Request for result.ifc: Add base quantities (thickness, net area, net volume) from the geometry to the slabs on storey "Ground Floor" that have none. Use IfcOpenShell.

First a look at what the model holds.

```python
import ifcopenshell
import ifcopenshell.util.element
import ifcopenshell.util.unit

model = ifcopenshell.open("result.ifc")
print(model.schema)
for unit_type in ("LENGTHUNIT", "AREAUNIT", "VOLUMEUNIT"):
    print(unit_type, ifcopenshell.util.unit.calculate_unit_scale(model, unit_type))
storey = next(s for s in model.by_type("IfcBuildingStorey") if s.Name == "Ground Floor")
slabs = [e for e in ifcopenshell.util.element.get_decomposition(storey) if e.is_a("IfcSlab")]
for e in sorted(slabs, key=lambda e: e.id()):
    print(e.id(), e.is_a(), e.Name, list(ifcopenshell.util.element.get_psets(e, qtos_only=True)), sep=" | ")
```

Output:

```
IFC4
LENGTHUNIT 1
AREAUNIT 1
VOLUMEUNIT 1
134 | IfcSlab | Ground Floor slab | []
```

```python
import ifcopenshell
import ifcopenshell.api.pset
import ifcopenshell.geom
import ifcopenshell.util.element
import ifcopenshell.util.shape
import ifcopenshell.util.unit

model = ifcopenshell.open("result.ifc")
unit_scale = ifcopenshell.util.unit.calculate_unit_scale(model)
area_scale = ifcopenshell.util.unit.calculate_unit_scale(model, "AREAUNIT")
volume_scale = ifcopenshell.util.unit.calculate_unit_scale(model, "VOLUMEUNIT")
settings = ifcopenshell.geom.settings()

storey = next(s for s in model.by_type("IfcBuildingStorey") if s.Name == "Ground Floor")
slabs = [e for e in ifcopenshell.util.element.get_decomposition(storey) if e.is_a("IfcSlab")]

for e in sorted(slabs, key=lambda e: e.id()):
    if ifcopenshell.util.element.get_psets(e, qtos_only=True, should_inherit=False):
        continue
    # Geometry comes back in metres, in the element's own axes.
    shape = ifcopenshell.geom.create_shape(settings, e)
    values = {
        "Width": ifcopenshell.util.shape.get_z(shape.geometry) / unit_scale,
        "NetArea": ifcopenshell.util.shape.get_footprint_area(shape.geometry) / area_scale,
        "NetVolume": ifcopenshell.util.shape.get_volume(shape.geometry) / volume_scale,
    }
    qto = ifcopenshell.api.pset.add_qto(model, product=e, name="Qto_SlabBaseQuantities")
    ifcopenshell.api.pset.edit_qto(model, qto=qto, properties=values)
    print(e.id(), {k: round(v, 3) for k, v in values.items()})

model.write("result-out.ifc")
```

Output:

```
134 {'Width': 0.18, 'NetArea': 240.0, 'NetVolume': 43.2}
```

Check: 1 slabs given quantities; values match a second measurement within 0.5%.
